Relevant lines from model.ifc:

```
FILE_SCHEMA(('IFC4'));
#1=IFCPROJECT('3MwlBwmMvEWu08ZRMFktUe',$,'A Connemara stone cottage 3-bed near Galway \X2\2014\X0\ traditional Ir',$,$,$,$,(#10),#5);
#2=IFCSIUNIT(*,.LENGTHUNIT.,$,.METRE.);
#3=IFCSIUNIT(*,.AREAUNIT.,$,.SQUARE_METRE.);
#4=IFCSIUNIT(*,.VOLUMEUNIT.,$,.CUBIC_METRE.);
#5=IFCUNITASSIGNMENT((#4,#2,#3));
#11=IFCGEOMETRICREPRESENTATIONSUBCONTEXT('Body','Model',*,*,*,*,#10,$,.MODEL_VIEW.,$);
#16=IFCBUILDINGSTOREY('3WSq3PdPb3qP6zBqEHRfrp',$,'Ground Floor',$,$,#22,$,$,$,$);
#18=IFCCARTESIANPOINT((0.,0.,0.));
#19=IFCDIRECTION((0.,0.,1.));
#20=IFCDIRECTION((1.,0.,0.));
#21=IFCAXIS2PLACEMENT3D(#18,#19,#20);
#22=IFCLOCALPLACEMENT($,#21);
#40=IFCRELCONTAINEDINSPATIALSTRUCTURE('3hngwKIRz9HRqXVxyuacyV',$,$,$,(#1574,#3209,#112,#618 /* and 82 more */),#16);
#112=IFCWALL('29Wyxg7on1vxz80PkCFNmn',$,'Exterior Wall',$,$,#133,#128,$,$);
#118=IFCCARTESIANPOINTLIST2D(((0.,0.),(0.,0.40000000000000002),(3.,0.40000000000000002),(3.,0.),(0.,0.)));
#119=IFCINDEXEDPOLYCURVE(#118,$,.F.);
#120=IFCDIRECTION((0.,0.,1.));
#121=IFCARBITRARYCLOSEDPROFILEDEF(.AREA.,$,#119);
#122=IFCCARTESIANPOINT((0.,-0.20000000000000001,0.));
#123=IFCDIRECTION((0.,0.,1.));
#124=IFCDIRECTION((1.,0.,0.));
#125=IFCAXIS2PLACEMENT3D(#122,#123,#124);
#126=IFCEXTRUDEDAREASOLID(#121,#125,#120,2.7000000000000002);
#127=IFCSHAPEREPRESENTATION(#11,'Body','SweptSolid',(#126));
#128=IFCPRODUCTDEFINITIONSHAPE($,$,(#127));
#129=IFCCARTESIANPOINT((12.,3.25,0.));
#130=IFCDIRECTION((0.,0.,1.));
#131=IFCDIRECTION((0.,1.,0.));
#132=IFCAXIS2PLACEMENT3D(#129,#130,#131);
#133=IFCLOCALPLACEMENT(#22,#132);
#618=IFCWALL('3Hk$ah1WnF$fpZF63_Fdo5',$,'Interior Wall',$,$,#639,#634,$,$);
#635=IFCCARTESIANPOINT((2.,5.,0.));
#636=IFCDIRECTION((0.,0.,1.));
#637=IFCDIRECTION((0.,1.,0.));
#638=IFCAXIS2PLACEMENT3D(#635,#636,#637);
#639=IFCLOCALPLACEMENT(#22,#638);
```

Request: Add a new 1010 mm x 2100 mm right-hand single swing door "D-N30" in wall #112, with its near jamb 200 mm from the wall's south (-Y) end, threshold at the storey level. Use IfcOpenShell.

```python
import numpy as np
import ifcopenshell
import ifcopenshell.api.feature
import ifcopenshell.api.geometry
import ifcopenshell.api.root
import ifcopenshell.api.spatial
import ifcopenshell.geom
import ifcopenshell.util.element
import ifcopenshell.util.placement
import ifcopenshell.util.representation
import ifcopenshell.util.shape
import ifcopenshell.util.unit

model = ifcopenshell.open("model.ifc")
unit_scale = ifcopenshell.util.unit.calculate_unit_scale(model)
settings = ifcopenshell.geom.settings()


def volume(element):
    """Net volume in cubic metres, openings subtracted."""
    shape = ifcopenshell.geom.create_shape(settings, element)
    return ifcopenshell.util.shape.get_volume(shape.geometry)


wall = model.by_guid("29Wyxg7on1vxz80PkCFNmn")
storey = ifcopenshell.util.element.get_container(wall, ifc_class="IfcBuildingStorey")
context = ifcopenshell.util.representation.get_context(model, "Model", "Body", "MODEL_VIEW")
before = volume(wall)

width, height, from_end, sill = 1.01, 2.1, 0.2, 0.0  # metres

# The wall runs along its own X axis, and the end named is its -X end.
wall_shape = ifcopenshell.geom.create_shape(settings, wall)
x, y, z = ifcopenshell.util.shape.get_vertices(wall_shape.geometry).T
start = x.min() + from_end
face, thickness = float(y.min()), float(y.max() - y.min())
wall_matrix = ifcopenshell.util.placement.get_local_placement(wall.ObjectPlacement)
level = ifcopenshell.util.placement.get_local_placement(storey.ObjectPlacement)[2, 3]


def in_wall(x, y):
    """Placement at x, y metres in the wall's axes, at sill height."""
    matrix = wall_matrix.copy()
    matrix[:, 3] = wall_matrix @ np.array([x / unit_scale, y / unit_scale, 0.0, 1.0])
    matrix[2, 3] = level + sill / unit_scale
    return matrix


# Opening: a box that overshoots both wall faces by 50 mm.
opening = ifcopenshell.api.root.create_entity(model, ifc_class="IfcOpeningElement", predefined_type="OPENING")
box = ifcopenshell.api.geometry.add_wall_representation(
    model, context=context, length=width, height=height, thickness=thickness + 0.1
)
ifcopenshell.api.geometry.assign_representation(model, product=opening, representation=box)
ifcopenshell.api.geometry.edit_object_placement(model, product=opening, matrix=in_wall(start, face - 0.05), is_si=False)
ifcopenshell.api.feature.add_feature(model, feature=opening, element=wall)

door = ifcopenshell.api.root.create_entity(model, ifc_class="IfcDoor", name="D-N30", predefined_type="DOOR")
door.OverallWidth, door.OverallHeight = width / unit_scale, height / unit_scale
door.OperationType = "SINGLE_SWING_RIGHT"
body = ifcopenshell.api.geometry.add_door_representation(
    model,
    context=context,
    overall_width=door.OverallWidth,
    overall_height=door.OverallHeight,
    operation_type="SINGLE_SWING_RIGHT",
    lining_properties={"LiningDepth": thickness / unit_scale, "ThresholdDepth": thickness / unit_scale},
)
ifcopenshell.api.geometry.assign_representation(model, product=door, representation=body)
ifcopenshell.api.spatial.assign_container(model, products=[door], relating_structure=storey)
ifcopenshell.api.feature.add_filling(model, opening=opening, element=door)

# The lining spans the wall, so the door starts at the wall face.
ifcopenshell.api.geometry.edit_object_placement(model, product=door, matrix=in_wall(start, face), is_si=False)

after = volume(wall)

print(f"wall volume {before:.3f} -> {after:.3f} m3")

model.write("model_rev.ifc")
```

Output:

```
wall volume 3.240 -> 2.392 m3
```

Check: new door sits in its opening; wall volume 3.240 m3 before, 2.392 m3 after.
